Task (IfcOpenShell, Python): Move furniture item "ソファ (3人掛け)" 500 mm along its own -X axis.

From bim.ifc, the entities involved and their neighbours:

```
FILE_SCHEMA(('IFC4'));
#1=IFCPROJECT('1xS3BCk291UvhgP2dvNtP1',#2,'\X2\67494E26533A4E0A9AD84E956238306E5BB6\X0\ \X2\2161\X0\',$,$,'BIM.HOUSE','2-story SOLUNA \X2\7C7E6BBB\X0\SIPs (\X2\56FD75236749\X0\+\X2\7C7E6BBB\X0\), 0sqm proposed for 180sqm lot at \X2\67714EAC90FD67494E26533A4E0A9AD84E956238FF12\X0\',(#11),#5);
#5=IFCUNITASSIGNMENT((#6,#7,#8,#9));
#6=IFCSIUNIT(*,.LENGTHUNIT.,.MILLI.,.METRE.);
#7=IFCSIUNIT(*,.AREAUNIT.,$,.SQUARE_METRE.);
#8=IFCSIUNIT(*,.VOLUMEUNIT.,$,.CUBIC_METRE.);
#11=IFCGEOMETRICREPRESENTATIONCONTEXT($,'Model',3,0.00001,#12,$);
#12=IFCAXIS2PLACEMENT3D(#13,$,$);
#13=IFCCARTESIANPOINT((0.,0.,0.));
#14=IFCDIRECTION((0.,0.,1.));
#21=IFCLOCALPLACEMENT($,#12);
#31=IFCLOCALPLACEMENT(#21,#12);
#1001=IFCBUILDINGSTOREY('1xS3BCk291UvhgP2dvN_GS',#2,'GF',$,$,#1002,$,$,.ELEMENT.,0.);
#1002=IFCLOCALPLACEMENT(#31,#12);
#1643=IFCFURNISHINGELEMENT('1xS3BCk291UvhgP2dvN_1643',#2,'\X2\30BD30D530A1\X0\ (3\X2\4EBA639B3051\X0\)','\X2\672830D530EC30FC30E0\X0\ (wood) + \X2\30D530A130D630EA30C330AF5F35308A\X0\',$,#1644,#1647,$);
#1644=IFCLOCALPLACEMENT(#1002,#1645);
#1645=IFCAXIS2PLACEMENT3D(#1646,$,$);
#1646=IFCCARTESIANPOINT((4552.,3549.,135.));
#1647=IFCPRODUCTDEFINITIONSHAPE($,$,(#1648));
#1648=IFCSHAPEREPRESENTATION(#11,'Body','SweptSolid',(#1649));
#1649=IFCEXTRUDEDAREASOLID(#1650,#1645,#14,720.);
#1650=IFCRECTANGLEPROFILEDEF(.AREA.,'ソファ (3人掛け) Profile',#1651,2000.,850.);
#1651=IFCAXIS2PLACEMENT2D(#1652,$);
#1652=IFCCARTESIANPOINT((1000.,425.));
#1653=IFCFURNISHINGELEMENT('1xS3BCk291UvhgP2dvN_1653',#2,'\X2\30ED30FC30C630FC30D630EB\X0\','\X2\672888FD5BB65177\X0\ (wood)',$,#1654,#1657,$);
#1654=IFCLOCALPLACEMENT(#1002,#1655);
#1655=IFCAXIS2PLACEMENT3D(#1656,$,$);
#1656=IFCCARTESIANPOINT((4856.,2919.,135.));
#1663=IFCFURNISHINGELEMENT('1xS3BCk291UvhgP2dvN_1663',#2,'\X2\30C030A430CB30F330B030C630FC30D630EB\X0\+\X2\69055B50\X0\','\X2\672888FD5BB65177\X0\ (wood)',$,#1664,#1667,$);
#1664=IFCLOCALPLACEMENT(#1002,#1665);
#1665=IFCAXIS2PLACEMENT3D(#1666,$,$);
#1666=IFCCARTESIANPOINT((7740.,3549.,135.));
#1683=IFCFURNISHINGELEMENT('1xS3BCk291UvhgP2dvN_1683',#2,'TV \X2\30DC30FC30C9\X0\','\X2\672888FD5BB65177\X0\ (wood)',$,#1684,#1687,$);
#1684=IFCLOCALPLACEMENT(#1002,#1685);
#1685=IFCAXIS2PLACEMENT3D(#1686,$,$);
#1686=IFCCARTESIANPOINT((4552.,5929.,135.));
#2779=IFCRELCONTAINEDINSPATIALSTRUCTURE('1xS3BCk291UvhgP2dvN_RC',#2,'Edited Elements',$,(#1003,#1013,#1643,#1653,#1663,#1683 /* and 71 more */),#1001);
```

```python
import ifcopenshell
import ifcopenshell.api.geometry
import ifcopenshell.util.placement

model = ifcopenshell.open("bim.ifc")

item = model.by_guid("1xS3BCk291UvhgP2dvN_1643")
matrix = ifcopenshell.util.placement.get_local_placement(item.ObjectPlacement)
matrix[:3, 3] -= matrix[:3, 0] * 500.0
ifcopenshell.api.geometry.edit_object_placement(model, product=item, matrix=matrix, is_si=False)

print(ifcopenshell.util.placement.get_local_placement(item.ObjectPlacement).round(3) + 0.0)

model.write("bim_updated.ifc")
```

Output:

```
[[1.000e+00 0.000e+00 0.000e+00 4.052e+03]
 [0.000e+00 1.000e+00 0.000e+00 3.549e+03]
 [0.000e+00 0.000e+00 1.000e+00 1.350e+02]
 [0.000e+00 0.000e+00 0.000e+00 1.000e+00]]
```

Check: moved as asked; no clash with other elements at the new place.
